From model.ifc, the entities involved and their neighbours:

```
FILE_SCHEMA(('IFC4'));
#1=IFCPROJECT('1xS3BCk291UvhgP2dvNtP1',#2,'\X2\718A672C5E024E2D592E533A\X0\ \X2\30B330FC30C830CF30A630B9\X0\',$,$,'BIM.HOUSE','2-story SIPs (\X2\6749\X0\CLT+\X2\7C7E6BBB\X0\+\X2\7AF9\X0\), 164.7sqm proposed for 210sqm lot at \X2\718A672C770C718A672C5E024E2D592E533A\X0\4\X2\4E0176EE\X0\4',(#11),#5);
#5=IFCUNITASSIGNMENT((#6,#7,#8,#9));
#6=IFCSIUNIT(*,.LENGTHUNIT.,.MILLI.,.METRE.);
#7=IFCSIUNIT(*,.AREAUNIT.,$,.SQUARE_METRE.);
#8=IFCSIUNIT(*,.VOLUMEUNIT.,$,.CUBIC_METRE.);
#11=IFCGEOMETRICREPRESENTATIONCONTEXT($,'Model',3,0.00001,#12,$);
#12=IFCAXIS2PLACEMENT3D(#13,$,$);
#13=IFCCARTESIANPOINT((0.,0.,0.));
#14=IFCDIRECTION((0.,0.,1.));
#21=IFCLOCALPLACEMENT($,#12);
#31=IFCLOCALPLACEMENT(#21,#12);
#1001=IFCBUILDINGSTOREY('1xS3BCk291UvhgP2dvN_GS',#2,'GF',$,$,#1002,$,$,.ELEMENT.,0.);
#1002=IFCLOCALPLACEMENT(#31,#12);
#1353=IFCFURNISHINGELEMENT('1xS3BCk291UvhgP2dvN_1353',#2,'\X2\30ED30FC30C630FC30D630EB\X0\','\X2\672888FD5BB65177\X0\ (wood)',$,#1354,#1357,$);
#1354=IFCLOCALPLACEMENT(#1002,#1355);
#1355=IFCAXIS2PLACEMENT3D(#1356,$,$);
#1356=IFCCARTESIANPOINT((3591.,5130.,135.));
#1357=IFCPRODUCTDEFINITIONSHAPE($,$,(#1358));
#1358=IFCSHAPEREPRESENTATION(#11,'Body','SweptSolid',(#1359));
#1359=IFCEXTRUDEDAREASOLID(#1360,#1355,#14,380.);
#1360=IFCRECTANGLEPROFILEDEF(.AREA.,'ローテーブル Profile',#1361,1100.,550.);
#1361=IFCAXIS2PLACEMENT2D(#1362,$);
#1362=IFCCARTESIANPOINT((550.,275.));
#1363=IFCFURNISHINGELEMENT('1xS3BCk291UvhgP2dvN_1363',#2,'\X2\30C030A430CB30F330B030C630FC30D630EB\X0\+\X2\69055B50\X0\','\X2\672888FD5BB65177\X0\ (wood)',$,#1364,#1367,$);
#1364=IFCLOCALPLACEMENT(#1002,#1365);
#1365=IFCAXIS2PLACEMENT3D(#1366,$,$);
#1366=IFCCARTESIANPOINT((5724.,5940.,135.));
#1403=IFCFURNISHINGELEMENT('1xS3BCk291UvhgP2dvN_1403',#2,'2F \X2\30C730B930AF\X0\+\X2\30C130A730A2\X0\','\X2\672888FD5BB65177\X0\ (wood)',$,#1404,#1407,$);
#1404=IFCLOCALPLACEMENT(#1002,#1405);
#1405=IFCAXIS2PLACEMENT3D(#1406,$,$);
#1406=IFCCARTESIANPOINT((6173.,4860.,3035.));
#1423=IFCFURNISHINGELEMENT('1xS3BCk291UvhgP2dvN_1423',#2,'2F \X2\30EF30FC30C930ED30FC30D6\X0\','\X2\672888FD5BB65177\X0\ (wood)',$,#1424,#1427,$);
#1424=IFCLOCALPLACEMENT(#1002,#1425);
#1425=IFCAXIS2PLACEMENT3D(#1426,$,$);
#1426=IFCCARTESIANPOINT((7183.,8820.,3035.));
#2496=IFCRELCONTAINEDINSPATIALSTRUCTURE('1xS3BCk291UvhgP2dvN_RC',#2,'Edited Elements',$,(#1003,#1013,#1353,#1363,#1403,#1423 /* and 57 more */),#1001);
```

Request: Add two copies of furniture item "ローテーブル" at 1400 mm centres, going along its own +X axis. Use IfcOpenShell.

```python
import ifcopenshell
import ifcopenshell.api.geometry
import ifcopenshell.api.root
import ifcopenshell.util.element
import ifcopenshell.util.placement

model = ifcopenshell.open("model.ifc")


def reuse_history(source, copy):
    """copy_class also copies each property set's owner history, people and application; keep the originals."""
    for rel in copy.IsDefinedBy:
        if rel.is_a("IfcRelDefinesByProperties") and (history := rel.RelatingPropertyDefinition.OwnerHistory):
            rel.RelatingPropertyDefinition.OwnerHistory = source.OwnerHistory
            ifcopenshell.util.element.remove_deep2(model, history)


source = model.by_guid("1xS3BCk291UvhgP2dvN_1353")
base = ifcopenshell.util.placement.get_local_placement(source.ObjectPlacement)
step = base[:3, 0] * 1400.0

for i in range(1, 3):
    copy = ifcopenshell.api.root.copy_class(model, product=source)
    copy.Representation = ifcopenshell.util.element.copy_deep(
        model, source.Representation, exclude=["IfcGeometricRepresentationContext", "IfcRepresentationMap"]
    )
    reuse_history(source, copy)
    matrix = base.copy()
    matrix[:3, 3] += i * step
    print("added at", matrix[:3, 3].round(3) + 0.0)
    ifcopenshell.api.geometry.edit_object_placement(model, product=copy, matrix=matrix, is_si=False)

model.write("model_v2.ifc")
```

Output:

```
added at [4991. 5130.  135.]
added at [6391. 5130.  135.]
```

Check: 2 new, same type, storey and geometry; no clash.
